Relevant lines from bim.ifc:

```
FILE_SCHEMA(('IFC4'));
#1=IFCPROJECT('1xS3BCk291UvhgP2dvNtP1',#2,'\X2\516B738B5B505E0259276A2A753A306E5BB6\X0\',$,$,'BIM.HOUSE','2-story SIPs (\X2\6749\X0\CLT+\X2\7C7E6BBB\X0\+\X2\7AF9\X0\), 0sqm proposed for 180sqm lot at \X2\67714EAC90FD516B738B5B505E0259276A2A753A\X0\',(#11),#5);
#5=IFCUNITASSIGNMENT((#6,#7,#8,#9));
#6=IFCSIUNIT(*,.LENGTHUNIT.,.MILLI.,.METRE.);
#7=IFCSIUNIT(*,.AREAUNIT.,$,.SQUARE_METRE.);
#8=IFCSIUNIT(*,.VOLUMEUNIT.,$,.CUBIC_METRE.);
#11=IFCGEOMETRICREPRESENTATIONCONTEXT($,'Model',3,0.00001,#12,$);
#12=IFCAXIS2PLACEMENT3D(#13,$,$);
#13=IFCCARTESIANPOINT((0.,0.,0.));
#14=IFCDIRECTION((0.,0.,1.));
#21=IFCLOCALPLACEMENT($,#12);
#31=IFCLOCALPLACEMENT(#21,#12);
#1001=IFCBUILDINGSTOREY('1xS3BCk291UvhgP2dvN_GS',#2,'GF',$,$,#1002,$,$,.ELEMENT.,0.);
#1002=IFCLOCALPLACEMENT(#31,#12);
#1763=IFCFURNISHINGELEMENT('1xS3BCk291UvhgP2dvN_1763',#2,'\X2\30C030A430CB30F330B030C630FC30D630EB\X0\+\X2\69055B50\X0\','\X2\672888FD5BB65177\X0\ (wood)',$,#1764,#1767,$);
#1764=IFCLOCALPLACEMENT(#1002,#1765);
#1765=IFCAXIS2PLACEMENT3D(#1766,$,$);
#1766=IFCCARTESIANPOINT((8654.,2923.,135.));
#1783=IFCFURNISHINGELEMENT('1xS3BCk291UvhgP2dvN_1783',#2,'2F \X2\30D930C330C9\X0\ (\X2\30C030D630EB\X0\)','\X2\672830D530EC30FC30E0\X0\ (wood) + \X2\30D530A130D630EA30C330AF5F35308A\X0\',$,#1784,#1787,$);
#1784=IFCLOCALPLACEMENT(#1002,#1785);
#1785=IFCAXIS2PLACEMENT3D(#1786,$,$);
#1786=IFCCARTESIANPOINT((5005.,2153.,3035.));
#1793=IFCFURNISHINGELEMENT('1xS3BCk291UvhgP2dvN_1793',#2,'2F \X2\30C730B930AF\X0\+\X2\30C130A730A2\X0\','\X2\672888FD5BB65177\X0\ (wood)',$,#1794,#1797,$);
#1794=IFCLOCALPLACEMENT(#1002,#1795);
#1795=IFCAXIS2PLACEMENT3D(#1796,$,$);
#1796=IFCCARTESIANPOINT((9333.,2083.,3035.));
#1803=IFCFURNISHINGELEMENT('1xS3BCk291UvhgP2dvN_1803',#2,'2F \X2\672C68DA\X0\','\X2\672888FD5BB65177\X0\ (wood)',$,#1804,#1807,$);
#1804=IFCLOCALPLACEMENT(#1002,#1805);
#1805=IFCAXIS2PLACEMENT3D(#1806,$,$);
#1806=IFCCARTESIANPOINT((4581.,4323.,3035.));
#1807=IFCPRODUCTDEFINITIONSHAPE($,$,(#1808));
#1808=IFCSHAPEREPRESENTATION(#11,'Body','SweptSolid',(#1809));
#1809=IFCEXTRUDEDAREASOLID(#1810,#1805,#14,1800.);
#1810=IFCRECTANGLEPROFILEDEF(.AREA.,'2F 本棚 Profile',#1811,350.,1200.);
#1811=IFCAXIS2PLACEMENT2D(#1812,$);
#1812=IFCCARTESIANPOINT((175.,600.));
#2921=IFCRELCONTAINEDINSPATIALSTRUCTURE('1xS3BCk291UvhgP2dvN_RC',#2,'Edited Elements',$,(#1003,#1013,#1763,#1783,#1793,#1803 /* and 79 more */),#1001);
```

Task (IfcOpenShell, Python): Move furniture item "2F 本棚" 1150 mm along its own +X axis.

```python
import ifcopenshell
import ifcopenshell.api.geometry
import ifcopenshell.util.placement

model = ifcopenshell.open("bim.ifc")

item = model.by_guid("1xS3BCk291UvhgP2dvN_1803")
matrix = ifcopenshell.util.placement.get_local_placement(item.ObjectPlacement)
matrix[:3, 3] += matrix[:3, 0] * 1150.0
ifcopenshell.api.geometry.edit_object_placement(model, product=item, matrix=matrix, is_si=False)

print(ifcopenshell.util.placement.get_local_placement(item.ObjectPlacement).round(3) + 0.0)

model.write("bim_rev.ifc")
```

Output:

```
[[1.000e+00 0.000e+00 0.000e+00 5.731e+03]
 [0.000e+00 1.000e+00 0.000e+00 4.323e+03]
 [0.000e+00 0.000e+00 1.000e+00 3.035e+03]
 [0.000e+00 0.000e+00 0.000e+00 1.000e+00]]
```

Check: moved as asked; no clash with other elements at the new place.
